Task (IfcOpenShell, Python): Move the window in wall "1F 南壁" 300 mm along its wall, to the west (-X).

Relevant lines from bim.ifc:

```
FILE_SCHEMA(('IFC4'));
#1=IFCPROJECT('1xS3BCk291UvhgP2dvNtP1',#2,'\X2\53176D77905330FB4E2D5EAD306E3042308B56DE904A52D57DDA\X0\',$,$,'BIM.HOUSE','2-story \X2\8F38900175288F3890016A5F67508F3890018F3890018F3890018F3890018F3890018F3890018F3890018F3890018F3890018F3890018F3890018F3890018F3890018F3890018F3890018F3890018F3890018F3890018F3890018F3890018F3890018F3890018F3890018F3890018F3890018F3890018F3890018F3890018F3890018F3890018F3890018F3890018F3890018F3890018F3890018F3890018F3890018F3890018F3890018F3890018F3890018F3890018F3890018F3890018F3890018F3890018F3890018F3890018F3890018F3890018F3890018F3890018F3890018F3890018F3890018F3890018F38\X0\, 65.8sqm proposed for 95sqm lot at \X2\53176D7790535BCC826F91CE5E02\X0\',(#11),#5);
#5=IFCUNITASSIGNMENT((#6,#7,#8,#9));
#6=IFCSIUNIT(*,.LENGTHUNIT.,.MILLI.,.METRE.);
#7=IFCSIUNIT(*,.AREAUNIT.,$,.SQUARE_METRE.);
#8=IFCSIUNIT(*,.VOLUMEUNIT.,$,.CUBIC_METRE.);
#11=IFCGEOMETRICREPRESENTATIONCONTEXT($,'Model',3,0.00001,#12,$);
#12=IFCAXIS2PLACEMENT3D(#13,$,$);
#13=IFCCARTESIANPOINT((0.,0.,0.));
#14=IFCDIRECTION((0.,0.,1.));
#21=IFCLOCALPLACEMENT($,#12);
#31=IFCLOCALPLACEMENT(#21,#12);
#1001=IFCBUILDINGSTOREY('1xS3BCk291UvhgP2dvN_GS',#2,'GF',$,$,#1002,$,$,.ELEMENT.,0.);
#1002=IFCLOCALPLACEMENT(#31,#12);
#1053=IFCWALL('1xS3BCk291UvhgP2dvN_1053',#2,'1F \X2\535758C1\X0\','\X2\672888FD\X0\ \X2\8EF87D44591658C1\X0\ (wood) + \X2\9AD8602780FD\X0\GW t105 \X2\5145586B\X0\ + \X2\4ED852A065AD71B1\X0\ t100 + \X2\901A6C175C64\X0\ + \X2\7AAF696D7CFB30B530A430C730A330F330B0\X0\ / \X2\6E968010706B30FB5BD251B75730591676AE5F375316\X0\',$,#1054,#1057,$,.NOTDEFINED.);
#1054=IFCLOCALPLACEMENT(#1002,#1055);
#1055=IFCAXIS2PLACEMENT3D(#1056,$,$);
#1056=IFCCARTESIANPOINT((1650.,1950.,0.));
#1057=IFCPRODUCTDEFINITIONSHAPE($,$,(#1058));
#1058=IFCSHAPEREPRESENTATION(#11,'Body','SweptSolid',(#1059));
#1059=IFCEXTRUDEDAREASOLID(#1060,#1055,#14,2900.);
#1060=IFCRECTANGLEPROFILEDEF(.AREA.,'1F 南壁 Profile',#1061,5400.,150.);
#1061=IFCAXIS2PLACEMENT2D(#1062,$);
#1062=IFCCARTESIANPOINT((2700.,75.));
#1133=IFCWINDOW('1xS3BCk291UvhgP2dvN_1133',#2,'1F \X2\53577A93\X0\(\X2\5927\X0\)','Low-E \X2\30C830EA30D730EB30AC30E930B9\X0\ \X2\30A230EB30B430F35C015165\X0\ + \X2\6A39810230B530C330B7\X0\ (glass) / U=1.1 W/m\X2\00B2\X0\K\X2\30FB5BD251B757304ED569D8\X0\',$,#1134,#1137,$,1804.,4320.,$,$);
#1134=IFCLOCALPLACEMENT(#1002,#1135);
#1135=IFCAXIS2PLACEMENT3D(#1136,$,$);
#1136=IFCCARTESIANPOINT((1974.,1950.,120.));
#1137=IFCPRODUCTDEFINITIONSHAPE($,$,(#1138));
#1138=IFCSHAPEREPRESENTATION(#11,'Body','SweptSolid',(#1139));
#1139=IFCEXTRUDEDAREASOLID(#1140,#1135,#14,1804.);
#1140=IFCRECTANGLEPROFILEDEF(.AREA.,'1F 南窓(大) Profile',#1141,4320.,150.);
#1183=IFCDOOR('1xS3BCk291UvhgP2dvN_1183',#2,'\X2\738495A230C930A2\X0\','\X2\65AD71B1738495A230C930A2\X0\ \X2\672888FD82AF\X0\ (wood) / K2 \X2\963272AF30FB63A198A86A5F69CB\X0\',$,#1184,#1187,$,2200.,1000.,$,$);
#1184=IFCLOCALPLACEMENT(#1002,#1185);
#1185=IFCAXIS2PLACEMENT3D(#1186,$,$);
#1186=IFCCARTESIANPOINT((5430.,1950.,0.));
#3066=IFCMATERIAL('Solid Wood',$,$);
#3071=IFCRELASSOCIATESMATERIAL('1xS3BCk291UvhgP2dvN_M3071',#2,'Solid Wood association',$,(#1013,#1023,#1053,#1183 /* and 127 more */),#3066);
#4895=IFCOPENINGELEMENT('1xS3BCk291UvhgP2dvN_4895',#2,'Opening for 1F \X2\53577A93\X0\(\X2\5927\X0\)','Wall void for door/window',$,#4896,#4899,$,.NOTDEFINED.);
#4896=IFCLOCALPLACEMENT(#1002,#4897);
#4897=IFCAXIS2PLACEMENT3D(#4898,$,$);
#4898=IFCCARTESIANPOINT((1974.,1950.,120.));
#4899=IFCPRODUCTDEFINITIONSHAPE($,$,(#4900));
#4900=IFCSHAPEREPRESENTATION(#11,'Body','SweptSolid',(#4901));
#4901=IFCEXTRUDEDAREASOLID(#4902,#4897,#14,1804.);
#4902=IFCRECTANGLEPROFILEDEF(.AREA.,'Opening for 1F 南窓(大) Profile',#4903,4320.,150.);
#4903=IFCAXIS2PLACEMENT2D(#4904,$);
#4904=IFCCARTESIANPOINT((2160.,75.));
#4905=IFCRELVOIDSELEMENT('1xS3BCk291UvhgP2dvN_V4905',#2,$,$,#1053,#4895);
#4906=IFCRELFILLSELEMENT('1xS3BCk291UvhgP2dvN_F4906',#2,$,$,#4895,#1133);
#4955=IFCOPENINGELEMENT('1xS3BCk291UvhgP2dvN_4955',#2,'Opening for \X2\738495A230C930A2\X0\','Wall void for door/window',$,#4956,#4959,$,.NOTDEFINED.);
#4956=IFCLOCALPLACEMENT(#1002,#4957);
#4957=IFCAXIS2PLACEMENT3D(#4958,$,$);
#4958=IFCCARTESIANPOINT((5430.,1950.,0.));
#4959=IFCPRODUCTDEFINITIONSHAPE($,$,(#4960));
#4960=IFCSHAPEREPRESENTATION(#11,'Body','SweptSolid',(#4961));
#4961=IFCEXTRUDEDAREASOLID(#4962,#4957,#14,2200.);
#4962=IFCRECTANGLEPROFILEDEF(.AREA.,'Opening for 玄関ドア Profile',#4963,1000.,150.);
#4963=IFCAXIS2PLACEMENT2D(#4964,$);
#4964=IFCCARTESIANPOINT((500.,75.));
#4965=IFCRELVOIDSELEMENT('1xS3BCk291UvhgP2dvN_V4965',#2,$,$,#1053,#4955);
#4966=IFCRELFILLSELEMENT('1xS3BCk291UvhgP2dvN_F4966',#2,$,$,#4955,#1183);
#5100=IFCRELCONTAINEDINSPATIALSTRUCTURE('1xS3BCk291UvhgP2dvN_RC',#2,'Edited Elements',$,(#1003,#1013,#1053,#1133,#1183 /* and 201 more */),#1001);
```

```python
import ifcopenshell
import ifcopenshell.api.geometry
import ifcopenshell.util.placement
import ifcopenshell.util.unit

model = ifcopenshell.open("bim.ifc")
unit_scale = ifcopenshell.util.unit.calculate_unit_scale(model)

window = model.by_guid("1xS3BCk291UvhgP2dvN_1133")
opening = window.FillsVoids[0].RelatingOpeningElement
wall = opening.VoidsElements[0].RelatingBuildingElement

wall_matrix = ifcopenshell.util.placement.get_local_placement(wall.ObjectPlacement)
shift = wall_matrix[:3, 0] * -0.3 / unit_scale
before = ifcopenshell.util.placement.get_local_placement(window.ObjectPlacement)[:3, 3].copy()

# The window is not placed relative to its opening, so move both.
for product in (opening, window):
    matrix = ifcopenshell.util.placement.get_local_placement(product.ObjectPlacement)
    matrix[:3, 3] += shift
    ifcopenshell.api.geometry.edit_object_placement(model, product=product, matrix=matrix, is_si=False)

after = ifcopenshell.util.placement.get_local_placement(window.ObjectPlacement)[:3, 3]
print("window moved by", (after - before).round(3) + 0.0)

model.write("bim_v2.ifc")
```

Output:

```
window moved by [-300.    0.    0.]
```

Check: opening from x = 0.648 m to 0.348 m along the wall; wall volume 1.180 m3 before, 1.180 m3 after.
